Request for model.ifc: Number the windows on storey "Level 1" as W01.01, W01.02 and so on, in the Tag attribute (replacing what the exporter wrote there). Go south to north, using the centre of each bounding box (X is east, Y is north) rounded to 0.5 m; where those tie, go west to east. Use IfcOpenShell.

First a look at what the model holds.

```python
import ifcopenshell
import ifcopenshell.util.element
import ifcopenshell.util.placement

model = ifcopenshell.open("model.ifc")
print(model.schema)
storey = next(s for s in model.by_type("IfcBuildingStorey") if s.Name == "Level 1")
windows = [e for e in ifcopenshell.util.element.get_decomposition(storey) if e.is_a("IfcWindow")]
for e in sorted(windows, key=lambda e: e.id()):
    origin = ifcopenshell.util.placement.get_local_placement(e.ObjectPlacement)[:3, 3]
    print(e.id(), e.Tag, e.Name, origin.round(2) + 0.0, sep=" | ")
```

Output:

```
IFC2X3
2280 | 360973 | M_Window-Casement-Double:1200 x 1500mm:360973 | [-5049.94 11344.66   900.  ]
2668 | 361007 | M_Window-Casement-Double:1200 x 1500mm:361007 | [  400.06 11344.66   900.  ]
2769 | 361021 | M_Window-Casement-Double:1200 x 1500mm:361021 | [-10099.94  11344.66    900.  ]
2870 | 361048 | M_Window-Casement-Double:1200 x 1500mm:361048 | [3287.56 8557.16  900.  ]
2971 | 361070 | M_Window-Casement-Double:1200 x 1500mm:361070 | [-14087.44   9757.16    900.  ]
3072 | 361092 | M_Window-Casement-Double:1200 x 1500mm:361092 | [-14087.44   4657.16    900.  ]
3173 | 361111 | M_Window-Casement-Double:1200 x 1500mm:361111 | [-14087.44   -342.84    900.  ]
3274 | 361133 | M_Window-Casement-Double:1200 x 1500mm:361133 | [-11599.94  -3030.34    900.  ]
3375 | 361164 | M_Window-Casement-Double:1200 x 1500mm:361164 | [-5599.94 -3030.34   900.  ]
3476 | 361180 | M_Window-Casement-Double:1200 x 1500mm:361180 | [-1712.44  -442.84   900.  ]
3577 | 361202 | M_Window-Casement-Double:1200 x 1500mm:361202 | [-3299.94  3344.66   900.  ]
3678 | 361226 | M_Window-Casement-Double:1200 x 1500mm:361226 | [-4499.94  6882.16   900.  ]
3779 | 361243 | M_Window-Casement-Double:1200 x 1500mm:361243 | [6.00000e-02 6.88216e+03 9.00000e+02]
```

```python
import ifcopenshell
import ifcopenshell.geom
import ifcopenshell.util.element
import ifcopenshell.util.shape

model = ifcopenshell.open("model.ifc")
settings = ifcopenshell.geom.settings()
settings.set("use-world-coords", True)


def centre(element):
    shape = ifcopenshell.geom.create_shape(settings, element)
    return ifcopenshell.util.shape.get_bbox_centroid(shape.geometry)


storey = next(s for s in model.by_type("IfcBuildingStorey") if s.Name == "Level 1")
windows = [e for e in ifcopenshell.util.element.get_decomposition(storey) if e.is_a("IfcWindow")]

# Insertion points can sit at a corner or the storey origin, so sort by the geometry (in metres).
centres = {e: centre(e) for e in windows}
windows.sort(key=lambda e: (round(centres[e][1] / 0.5), centres[e][0]))

for i, e in enumerate(windows, start=1):
    number = f"W01.{i:02d}"
    e.Tag = number
    print(e.id(), number)

model.write("model_v2.ifc")
```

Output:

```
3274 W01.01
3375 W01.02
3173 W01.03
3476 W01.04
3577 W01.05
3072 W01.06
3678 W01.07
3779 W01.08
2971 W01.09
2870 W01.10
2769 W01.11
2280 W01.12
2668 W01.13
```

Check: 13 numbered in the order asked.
